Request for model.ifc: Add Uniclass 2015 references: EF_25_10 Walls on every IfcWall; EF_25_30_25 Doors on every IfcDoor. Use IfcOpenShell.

First a look at what the model holds.

```python
import ifcopenshell

model = ifcopenshell.open("model.ifc")
print(model.schema)
print("classifications:", [c.Name for c in model.by_type("IfcClassification")])
for ifc_class in ("IfcDoor", "IfcRoof", "IfcStair", "IfcWall", "IfcWindow"):
    print(ifc_class, len(model.by_type(ifc_class)))
```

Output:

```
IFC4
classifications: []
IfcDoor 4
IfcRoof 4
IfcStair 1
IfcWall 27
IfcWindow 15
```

```python
import ifcopenshell
import ifcopenshell.api.classification

model = ifcopenshell.open("model.ifc")

system = ifcopenshell.api.classification.add_classification(model, classification="Uniclass 2015")

codes = {
    "IfcWall": ("EF_25_10", "Walls"),
    "IfcDoor": ("EF_25_30_25", "Doors"),
}
for ifc_class, (code, name) in codes.items():
    products = model.by_type(ifc_class)
    ifcopenshell.api.classification.add_reference(
        model, products=products, classification=system, identification=code, name=name
    )
    print(code, len(products))

model.write("model-out.ifc")
```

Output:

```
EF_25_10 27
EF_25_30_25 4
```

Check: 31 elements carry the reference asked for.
